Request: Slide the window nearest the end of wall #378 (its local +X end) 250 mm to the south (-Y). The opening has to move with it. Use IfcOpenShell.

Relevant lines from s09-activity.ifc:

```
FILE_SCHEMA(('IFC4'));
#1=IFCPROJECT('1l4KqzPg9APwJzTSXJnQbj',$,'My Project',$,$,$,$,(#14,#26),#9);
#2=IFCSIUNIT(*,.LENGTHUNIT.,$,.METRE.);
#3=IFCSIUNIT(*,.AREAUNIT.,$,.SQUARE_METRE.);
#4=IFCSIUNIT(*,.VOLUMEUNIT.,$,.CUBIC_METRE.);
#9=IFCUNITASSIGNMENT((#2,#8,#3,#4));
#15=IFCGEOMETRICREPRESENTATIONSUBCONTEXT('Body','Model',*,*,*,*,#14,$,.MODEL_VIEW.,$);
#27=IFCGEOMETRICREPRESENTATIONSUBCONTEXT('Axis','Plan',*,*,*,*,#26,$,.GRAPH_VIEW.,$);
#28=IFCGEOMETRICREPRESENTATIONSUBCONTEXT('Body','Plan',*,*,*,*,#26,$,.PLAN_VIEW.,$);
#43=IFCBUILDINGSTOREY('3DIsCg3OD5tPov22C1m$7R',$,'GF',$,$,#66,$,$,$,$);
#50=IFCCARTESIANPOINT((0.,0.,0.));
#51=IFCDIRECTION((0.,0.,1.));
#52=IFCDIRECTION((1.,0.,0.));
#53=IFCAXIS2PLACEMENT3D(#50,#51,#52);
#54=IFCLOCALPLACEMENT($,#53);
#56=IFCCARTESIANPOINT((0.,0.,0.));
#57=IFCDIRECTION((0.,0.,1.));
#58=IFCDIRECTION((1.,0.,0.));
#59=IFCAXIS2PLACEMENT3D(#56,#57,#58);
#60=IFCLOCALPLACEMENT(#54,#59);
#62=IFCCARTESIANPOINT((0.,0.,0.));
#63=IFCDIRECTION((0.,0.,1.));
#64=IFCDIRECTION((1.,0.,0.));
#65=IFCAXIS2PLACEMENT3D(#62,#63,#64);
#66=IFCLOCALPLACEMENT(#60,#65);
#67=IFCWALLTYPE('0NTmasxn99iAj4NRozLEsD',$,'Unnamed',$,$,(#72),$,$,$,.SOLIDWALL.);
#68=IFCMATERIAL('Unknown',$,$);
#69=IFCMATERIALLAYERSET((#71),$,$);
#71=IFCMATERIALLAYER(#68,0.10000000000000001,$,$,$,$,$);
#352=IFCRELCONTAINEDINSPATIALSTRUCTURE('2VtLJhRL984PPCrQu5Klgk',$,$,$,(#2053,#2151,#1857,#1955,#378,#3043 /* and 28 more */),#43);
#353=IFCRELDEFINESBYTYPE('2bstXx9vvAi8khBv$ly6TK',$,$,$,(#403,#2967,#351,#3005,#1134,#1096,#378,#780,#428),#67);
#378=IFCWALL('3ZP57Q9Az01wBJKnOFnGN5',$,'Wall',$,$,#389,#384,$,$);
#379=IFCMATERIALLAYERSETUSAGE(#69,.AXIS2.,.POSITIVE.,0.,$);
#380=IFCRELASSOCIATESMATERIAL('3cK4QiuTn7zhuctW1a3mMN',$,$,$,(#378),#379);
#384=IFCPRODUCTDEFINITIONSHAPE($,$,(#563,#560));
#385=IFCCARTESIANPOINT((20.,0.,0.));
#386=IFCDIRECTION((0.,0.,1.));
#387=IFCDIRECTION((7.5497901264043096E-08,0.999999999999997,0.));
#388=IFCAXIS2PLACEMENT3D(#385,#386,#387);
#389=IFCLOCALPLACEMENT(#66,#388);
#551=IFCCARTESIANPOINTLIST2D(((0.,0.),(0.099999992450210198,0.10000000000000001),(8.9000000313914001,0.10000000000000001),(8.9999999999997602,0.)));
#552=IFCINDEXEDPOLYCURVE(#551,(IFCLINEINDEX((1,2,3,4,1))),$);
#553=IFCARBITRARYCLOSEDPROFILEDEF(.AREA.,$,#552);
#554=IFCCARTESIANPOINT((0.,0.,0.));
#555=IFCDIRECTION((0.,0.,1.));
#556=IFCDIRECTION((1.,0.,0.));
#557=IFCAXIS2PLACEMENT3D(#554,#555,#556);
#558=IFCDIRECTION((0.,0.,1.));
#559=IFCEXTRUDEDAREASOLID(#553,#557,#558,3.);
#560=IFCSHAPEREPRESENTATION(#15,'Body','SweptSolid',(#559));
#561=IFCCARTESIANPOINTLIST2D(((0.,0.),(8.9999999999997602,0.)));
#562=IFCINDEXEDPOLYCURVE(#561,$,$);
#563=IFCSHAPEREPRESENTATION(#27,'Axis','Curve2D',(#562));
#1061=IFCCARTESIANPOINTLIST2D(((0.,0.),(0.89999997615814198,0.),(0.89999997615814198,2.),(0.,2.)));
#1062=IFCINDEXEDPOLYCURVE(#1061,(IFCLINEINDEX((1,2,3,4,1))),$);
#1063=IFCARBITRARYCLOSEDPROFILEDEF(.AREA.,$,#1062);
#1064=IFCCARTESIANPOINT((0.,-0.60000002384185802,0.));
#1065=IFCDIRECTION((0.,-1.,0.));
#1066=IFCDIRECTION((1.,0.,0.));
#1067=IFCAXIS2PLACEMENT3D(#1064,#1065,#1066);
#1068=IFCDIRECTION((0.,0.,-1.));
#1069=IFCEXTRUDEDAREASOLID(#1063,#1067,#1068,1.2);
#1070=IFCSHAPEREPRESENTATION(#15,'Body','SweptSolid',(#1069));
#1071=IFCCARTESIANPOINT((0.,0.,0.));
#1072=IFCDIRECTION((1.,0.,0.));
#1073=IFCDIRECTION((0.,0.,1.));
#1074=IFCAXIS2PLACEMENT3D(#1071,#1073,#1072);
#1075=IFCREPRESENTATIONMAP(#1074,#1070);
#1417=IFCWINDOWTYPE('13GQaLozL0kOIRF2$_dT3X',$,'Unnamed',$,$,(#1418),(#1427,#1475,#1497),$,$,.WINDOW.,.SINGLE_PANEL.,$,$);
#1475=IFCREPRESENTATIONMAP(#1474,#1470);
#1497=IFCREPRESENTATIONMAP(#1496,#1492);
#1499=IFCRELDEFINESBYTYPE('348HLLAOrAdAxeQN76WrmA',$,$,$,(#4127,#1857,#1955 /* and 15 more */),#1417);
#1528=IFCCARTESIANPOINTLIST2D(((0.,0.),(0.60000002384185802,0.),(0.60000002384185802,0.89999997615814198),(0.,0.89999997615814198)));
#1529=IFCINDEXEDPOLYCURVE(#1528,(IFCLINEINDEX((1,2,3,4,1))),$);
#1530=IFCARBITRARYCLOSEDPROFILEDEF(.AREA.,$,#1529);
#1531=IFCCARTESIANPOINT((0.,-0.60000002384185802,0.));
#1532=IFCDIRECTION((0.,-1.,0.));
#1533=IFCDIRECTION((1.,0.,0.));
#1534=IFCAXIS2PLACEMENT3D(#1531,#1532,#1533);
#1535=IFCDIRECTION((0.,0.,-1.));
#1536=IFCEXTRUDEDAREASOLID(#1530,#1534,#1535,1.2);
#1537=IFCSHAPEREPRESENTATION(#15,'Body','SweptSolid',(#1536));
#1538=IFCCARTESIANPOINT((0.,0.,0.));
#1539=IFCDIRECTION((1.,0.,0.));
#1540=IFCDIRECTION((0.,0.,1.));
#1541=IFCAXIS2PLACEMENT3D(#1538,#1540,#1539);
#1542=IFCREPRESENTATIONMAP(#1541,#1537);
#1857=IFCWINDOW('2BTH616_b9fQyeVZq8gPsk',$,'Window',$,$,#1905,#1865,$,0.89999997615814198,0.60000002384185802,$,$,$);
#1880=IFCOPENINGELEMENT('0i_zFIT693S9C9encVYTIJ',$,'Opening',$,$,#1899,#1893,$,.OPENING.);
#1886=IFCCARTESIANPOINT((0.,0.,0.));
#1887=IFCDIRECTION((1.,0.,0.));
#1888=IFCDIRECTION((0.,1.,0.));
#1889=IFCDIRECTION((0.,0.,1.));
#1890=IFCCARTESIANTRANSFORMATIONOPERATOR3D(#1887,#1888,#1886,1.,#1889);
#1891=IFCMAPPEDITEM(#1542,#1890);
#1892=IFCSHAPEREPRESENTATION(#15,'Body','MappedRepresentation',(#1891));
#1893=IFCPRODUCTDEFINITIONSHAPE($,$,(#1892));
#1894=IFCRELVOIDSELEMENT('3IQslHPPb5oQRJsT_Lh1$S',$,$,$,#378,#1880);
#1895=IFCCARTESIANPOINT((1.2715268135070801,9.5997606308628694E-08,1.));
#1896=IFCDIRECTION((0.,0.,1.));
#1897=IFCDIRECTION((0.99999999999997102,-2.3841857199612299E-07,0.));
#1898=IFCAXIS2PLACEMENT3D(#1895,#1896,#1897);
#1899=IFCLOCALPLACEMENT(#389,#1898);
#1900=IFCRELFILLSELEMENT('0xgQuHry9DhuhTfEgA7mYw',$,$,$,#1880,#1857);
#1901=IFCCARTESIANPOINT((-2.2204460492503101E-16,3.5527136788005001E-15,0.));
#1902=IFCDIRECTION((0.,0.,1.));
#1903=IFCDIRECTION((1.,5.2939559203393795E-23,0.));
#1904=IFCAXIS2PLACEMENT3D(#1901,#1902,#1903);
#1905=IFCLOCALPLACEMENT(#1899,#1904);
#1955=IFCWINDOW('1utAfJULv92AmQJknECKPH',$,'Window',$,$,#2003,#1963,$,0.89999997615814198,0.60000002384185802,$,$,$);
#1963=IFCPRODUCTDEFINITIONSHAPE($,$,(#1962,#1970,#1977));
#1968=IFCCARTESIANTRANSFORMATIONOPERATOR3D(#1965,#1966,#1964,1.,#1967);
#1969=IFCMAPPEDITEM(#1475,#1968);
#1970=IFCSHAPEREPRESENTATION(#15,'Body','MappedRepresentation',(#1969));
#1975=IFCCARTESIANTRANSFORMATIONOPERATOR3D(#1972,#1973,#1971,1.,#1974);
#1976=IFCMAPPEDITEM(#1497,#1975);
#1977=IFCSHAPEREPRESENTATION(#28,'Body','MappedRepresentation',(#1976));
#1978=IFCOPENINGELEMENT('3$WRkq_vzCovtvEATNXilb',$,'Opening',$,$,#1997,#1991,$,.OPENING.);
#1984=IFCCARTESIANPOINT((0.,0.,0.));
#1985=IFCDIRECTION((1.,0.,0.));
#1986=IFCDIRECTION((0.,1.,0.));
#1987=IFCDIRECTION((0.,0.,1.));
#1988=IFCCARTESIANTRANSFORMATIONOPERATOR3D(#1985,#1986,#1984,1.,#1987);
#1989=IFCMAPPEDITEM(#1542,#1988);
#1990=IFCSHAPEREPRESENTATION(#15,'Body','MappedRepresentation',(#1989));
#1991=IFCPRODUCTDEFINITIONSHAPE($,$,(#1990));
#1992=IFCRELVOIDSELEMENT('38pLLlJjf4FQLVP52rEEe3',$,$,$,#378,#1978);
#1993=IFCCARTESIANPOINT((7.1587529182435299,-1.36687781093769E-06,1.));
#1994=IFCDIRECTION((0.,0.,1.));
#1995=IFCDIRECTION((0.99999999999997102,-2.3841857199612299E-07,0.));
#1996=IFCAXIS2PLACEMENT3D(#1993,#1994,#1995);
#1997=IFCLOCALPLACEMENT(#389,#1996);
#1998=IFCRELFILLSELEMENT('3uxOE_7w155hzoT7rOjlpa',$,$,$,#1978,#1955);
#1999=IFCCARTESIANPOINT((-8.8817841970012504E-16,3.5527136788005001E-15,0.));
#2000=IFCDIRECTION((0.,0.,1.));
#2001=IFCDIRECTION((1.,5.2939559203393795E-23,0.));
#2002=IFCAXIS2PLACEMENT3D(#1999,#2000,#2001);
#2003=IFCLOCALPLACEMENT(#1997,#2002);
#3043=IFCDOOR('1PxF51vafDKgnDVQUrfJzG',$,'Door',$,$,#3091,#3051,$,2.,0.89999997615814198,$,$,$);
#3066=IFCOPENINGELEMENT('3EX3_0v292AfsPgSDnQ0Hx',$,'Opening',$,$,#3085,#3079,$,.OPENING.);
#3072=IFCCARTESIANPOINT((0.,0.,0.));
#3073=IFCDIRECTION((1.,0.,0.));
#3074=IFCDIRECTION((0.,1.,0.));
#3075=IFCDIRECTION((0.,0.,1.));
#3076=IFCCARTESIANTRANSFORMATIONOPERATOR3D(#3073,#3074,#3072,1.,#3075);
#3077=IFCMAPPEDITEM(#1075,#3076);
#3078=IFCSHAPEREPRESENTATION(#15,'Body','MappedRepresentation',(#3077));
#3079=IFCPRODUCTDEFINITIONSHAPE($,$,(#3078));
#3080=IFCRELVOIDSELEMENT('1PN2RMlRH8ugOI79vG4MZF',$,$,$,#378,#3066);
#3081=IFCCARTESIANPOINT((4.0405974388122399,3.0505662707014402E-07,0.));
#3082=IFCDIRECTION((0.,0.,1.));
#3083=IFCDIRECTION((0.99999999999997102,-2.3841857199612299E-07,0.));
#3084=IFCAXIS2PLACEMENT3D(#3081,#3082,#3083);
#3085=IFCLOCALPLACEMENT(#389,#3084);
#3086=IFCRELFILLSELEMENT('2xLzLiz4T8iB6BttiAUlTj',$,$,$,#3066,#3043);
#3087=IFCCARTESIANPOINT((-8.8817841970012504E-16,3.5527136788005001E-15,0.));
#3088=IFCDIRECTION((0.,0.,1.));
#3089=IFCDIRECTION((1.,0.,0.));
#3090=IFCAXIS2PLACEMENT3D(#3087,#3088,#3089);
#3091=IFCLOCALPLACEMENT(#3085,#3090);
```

```python
import ifcopenshell
import ifcopenshell.api.geometry
import ifcopenshell.util.placement
import ifcopenshell.util.unit

model = ifcopenshell.open("s09-activity.ifc")
unit_scale = ifcopenshell.util.unit.calculate_unit_scale(model)

window = model.by_id(1955)
opening = window.FillsVoids[0].RelatingOpeningElement
wall = opening.VoidsElements[0].RelatingBuildingElement

wall_matrix = ifcopenshell.util.placement.get_local_placement(wall.ObjectPlacement)
shift = wall_matrix[:3, 0] * -0.25 / unit_scale
before = ifcopenshell.util.placement.get_local_placement(window.ObjectPlacement)[:3, 3].copy()

# The window is placed relative to its opening, so it follows when the opening moves.
matrix = ifcopenshell.util.placement.get_local_placement(opening.ObjectPlacement)
matrix[:3, 3] += shift
ifcopenshell.api.geometry.edit_object_placement(
    model, product=opening, matrix=matrix, is_si=False, should_transform_children=True
)

after = ifcopenshell.util.placement.get_local_placement(window.ObjectPlacement)[:3, 3]
print("window moved by", (after - before).round(3) + 0.0)

model.write("s09-activity_rev.ifc")
```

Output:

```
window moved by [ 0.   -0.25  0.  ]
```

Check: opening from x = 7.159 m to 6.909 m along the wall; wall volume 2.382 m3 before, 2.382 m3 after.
